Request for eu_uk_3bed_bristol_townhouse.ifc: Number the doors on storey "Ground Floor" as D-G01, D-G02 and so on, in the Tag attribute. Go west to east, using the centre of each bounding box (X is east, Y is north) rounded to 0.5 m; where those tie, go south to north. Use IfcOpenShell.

First a look at what the model holds.

```python
import ifcopenshell
import ifcopenshell.util.element
import ifcopenshell.util.placement

model = ifcopenshell.open("eu_uk_3bed_bristol_townhouse.ifc")
print(model.schema)
storey = next(s for s in model.by_type("IfcBuildingStorey") if s.Name == "Ground Floor")
doors = [e for e in ifcopenshell.util.element.get_decomposition(storey) if e.is_a("IfcDoor")]
for e in sorted(doors, key=lambda e: e.id()):
    origin = ifcopenshell.util.placement.get_local_placement(e.ObjectPlacement)[:3, 3]
    print(e.id(), e.Tag, e.Name, origin.round(2) + 0.0, sep=" | ")
```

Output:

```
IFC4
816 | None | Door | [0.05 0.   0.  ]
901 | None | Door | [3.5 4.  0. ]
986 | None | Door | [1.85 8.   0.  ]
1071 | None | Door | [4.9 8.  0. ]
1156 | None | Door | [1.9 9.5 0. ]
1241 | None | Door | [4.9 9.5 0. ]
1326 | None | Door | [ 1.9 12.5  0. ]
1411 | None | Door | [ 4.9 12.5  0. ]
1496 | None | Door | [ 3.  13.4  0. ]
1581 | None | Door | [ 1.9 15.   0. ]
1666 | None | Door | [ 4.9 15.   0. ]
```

```python
import ifcopenshell
import ifcopenshell.geom
import ifcopenshell.util.element
import ifcopenshell.util.shape

model = ifcopenshell.open("eu_uk_3bed_bristol_townhouse.ifc")
settings = ifcopenshell.geom.settings()
settings.set("use-world-coords", True)


def centre(element):
    shape = ifcopenshell.geom.create_shape(settings, element)
    return ifcopenshell.util.shape.get_bbox_centroid(shape.geometry)


storey = next(s for s in model.by_type("IfcBuildingStorey") if s.Name == "Ground Floor")
doors = [e for e in ifcopenshell.util.element.get_decomposition(storey) if e.is_a("IfcDoor")]

# Insertion points can sit at a corner or the storey origin, so sort by the geometry (in metres).
centres = {e: centre(e) for e in doors}
doors.sort(key=lambda e: (round(centres[e][0] / 0.5), centres[e][1]))

for i, e in enumerate(doors, start=1):
    number = f"D-G{i:02d}"
    e.Tag = number
    print(e.id(), number)

model.write("eu_uk_3bed_bristol_townhouse_v2.ifc")
```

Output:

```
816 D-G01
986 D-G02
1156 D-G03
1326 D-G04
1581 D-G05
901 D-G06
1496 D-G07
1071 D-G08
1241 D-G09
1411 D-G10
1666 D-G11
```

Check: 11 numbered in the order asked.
